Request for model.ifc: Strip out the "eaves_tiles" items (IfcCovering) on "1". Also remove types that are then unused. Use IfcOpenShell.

First a look at what the model holds.

```python
import ifcopenshell
import ifcopenshell.util.element

model = ifcopenshell.open("model.ifc")
print(model.schema)
storey = next(s for s in model.by_type("IfcBuildingStorey") if s.Name == "1")
coverings = [e for e in ifcopenshell.util.element.get_decomposition(storey) if e.is_a("IfcCovering")]
seen = {}
for e in coverings:
    element_type = ifcopenshell.util.element.get_type(e)
    name = element_type.Name if element_type not in (None, e) else None
    seen[name] = seen.get(name, 0) + 1
for name, count in sorted(seen.items(), key=str):
    print(count, "x", name)
```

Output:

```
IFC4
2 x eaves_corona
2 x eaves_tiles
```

```python
import ifcopenshell
import ifcopenshell.api.root
import ifcopenshell.util.element

model = ifcopenshell.open("model.ifc")

storey = next(s for s in model.by_type("IfcBuildingStorey") if s.Name == "1")
coverings = [e for e in ifcopenshell.util.element.get_decomposition(storey) if e.is_a("IfcCovering")]
targets = [e for e in coverings if (t := ifcopenshell.util.element.get_type(e)) not in (None, e) and t.Name == "eaves_tiles"]
types = {ifcopenshell.util.element.get_type(e) for e in targets} - {None, *targets}

for e in targets:
    ifcopenshell.api.root.remove_product(model, product=e)
print(len(targets), "removed")

unused = [t for t in types if not ifcopenshell.util.element.get_types(t)]
for t in unused:
    ifcopenshell.api.root.remove_product(model, product=t)
print(len(unused), "unused types removed")

model.write("model_rev.ifc")
```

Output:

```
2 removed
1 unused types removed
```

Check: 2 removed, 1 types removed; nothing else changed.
